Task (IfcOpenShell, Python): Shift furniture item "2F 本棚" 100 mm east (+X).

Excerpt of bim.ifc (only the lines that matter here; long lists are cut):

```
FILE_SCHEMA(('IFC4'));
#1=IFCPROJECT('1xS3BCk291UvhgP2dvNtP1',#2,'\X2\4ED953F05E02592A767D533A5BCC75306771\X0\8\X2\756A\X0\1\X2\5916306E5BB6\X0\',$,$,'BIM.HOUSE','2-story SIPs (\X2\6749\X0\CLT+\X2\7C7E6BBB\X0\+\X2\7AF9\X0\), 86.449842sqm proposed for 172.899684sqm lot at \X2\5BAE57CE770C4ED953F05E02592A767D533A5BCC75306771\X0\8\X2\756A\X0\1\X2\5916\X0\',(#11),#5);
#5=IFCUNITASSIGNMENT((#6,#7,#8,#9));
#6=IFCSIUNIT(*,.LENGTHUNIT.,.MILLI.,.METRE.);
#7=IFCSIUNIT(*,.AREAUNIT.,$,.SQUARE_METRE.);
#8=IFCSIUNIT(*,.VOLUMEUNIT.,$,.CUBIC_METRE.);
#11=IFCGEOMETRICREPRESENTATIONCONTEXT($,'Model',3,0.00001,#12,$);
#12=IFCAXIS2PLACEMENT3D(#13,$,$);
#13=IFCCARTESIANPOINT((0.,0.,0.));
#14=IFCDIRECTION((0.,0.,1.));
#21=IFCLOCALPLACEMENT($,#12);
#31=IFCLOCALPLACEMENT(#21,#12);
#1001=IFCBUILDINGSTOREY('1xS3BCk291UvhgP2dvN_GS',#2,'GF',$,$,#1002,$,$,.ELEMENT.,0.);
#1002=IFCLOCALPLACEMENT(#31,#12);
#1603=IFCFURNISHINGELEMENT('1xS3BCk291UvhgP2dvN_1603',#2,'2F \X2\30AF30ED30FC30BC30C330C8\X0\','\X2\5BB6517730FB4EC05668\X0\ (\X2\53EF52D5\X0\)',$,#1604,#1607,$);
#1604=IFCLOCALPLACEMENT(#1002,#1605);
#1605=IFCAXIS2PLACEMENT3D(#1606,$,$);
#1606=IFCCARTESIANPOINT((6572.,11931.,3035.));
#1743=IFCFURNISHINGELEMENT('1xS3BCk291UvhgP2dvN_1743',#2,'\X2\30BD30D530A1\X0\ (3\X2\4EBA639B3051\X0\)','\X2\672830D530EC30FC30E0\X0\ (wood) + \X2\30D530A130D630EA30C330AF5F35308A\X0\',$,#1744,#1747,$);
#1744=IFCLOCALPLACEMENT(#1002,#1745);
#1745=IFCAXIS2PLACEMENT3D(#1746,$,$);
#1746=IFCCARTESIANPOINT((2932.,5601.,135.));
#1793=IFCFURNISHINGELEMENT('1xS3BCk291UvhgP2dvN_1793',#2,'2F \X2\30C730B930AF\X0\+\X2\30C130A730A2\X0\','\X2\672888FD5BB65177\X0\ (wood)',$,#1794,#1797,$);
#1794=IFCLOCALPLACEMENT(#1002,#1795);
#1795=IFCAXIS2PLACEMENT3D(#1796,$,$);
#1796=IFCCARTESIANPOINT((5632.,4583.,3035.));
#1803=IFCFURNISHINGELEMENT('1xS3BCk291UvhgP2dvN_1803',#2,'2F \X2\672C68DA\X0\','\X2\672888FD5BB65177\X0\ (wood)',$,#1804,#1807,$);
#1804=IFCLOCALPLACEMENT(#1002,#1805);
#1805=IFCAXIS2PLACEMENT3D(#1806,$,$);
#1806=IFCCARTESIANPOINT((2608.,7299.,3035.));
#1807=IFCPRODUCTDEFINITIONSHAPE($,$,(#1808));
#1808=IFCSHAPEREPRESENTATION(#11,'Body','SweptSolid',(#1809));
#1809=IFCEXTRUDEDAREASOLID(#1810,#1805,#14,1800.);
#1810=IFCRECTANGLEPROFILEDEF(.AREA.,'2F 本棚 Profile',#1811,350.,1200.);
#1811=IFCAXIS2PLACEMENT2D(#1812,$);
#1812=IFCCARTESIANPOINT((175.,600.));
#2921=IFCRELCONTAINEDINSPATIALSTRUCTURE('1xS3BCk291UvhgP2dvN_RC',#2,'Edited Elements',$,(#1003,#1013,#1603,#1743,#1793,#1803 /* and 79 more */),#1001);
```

```python
import ifcopenshell
import ifcopenshell.api.geometry
import ifcopenshell.util.placement

model = ifcopenshell.open("bim.ifc")

item = model.by_guid("1xS3BCk291UvhgP2dvN_1803")
matrix = ifcopenshell.util.placement.get_local_placement(item.ObjectPlacement)
matrix[0, 3] += 100.0
ifcopenshell.api.geometry.edit_object_placement(model, product=item, matrix=matrix, is_si=False)

print(ifcopenshell.util.placement.get_local_placement(item.ObjectPlacement).round(3) + 0.0)

model.write("bim_updated.ifc")
```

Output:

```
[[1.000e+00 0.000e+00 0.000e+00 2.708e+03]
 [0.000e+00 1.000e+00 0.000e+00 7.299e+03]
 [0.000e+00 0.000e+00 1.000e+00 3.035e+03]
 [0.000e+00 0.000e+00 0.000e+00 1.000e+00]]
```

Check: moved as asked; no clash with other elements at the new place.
